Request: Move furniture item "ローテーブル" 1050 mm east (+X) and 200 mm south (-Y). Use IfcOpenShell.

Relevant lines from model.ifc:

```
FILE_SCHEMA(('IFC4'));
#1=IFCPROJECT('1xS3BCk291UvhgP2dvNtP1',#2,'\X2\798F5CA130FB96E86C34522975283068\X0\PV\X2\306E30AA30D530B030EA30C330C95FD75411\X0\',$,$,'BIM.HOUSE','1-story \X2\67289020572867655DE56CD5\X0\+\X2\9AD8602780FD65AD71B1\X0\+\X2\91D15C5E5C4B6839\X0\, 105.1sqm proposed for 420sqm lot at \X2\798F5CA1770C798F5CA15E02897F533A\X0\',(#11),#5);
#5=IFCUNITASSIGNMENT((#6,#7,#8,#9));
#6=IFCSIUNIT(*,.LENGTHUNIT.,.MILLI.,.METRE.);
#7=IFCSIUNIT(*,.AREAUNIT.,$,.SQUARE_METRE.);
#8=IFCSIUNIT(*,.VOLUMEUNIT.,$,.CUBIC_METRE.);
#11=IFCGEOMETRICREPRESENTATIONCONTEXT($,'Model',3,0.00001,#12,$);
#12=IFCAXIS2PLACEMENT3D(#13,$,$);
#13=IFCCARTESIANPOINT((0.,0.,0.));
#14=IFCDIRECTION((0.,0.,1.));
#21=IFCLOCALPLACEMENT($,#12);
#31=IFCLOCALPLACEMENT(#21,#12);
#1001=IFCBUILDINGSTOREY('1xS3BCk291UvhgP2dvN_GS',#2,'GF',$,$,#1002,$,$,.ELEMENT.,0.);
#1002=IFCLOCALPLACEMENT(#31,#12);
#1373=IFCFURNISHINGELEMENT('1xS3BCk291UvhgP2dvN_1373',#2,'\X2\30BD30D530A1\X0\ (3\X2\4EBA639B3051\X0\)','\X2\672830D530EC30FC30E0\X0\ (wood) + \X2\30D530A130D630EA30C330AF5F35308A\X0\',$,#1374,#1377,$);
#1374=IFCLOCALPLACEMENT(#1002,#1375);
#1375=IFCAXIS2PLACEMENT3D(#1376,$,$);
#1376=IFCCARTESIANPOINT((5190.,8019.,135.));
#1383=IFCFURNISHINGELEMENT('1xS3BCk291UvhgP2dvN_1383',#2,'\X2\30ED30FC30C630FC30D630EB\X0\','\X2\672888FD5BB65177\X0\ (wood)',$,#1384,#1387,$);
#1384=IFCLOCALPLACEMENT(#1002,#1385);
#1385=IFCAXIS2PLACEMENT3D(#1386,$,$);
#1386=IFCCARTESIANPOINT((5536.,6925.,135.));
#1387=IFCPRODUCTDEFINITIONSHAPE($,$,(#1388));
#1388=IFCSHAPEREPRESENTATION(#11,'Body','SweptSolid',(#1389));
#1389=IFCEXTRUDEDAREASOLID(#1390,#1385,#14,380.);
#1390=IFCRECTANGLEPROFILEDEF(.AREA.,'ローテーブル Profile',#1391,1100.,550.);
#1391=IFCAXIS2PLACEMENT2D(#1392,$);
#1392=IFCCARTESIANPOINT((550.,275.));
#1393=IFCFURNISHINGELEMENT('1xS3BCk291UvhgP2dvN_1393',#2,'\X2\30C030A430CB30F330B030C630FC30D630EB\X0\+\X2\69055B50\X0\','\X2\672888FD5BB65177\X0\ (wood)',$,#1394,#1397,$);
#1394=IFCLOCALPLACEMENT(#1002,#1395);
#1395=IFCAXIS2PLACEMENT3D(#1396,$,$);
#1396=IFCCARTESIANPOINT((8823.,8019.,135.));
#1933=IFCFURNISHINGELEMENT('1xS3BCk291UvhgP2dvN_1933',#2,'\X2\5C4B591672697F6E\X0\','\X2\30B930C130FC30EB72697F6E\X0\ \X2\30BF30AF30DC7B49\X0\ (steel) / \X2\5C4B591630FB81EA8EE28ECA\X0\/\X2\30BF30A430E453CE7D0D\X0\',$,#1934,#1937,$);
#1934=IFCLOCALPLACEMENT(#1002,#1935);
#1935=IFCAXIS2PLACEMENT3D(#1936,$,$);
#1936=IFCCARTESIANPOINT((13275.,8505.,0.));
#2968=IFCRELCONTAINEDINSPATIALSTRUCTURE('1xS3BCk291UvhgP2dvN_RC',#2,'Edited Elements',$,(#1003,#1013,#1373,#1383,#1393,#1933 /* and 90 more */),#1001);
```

```python
import ifcopenshell
import ifcopenshell.api.geometry
import ifcopenshell.util.placement

model = ifcopenshell.open("model.ifc")

item = model.by_guid("1xS3BCk291UvhgP2dvN_1383")
matrix = ifcopenshell.util.placement.get_local_placement(item.ObjectPlacement)
matrix[0, 3] += 1050.0
matrix[1, 3] -= 200.0
ifcopenshell.api.geometry.edit_object_placement(model, product=item, matrix=matrix, is_si=False)

print(ifcopenshell.util.placement.get_local_placement(item.ObjectPlacement).round(3) + 0.0)

model.write("model_v2.ifc")
```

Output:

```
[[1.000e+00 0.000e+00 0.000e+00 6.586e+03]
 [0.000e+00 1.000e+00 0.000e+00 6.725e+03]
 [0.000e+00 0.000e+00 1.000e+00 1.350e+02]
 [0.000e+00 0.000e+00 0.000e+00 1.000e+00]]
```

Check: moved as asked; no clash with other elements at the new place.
